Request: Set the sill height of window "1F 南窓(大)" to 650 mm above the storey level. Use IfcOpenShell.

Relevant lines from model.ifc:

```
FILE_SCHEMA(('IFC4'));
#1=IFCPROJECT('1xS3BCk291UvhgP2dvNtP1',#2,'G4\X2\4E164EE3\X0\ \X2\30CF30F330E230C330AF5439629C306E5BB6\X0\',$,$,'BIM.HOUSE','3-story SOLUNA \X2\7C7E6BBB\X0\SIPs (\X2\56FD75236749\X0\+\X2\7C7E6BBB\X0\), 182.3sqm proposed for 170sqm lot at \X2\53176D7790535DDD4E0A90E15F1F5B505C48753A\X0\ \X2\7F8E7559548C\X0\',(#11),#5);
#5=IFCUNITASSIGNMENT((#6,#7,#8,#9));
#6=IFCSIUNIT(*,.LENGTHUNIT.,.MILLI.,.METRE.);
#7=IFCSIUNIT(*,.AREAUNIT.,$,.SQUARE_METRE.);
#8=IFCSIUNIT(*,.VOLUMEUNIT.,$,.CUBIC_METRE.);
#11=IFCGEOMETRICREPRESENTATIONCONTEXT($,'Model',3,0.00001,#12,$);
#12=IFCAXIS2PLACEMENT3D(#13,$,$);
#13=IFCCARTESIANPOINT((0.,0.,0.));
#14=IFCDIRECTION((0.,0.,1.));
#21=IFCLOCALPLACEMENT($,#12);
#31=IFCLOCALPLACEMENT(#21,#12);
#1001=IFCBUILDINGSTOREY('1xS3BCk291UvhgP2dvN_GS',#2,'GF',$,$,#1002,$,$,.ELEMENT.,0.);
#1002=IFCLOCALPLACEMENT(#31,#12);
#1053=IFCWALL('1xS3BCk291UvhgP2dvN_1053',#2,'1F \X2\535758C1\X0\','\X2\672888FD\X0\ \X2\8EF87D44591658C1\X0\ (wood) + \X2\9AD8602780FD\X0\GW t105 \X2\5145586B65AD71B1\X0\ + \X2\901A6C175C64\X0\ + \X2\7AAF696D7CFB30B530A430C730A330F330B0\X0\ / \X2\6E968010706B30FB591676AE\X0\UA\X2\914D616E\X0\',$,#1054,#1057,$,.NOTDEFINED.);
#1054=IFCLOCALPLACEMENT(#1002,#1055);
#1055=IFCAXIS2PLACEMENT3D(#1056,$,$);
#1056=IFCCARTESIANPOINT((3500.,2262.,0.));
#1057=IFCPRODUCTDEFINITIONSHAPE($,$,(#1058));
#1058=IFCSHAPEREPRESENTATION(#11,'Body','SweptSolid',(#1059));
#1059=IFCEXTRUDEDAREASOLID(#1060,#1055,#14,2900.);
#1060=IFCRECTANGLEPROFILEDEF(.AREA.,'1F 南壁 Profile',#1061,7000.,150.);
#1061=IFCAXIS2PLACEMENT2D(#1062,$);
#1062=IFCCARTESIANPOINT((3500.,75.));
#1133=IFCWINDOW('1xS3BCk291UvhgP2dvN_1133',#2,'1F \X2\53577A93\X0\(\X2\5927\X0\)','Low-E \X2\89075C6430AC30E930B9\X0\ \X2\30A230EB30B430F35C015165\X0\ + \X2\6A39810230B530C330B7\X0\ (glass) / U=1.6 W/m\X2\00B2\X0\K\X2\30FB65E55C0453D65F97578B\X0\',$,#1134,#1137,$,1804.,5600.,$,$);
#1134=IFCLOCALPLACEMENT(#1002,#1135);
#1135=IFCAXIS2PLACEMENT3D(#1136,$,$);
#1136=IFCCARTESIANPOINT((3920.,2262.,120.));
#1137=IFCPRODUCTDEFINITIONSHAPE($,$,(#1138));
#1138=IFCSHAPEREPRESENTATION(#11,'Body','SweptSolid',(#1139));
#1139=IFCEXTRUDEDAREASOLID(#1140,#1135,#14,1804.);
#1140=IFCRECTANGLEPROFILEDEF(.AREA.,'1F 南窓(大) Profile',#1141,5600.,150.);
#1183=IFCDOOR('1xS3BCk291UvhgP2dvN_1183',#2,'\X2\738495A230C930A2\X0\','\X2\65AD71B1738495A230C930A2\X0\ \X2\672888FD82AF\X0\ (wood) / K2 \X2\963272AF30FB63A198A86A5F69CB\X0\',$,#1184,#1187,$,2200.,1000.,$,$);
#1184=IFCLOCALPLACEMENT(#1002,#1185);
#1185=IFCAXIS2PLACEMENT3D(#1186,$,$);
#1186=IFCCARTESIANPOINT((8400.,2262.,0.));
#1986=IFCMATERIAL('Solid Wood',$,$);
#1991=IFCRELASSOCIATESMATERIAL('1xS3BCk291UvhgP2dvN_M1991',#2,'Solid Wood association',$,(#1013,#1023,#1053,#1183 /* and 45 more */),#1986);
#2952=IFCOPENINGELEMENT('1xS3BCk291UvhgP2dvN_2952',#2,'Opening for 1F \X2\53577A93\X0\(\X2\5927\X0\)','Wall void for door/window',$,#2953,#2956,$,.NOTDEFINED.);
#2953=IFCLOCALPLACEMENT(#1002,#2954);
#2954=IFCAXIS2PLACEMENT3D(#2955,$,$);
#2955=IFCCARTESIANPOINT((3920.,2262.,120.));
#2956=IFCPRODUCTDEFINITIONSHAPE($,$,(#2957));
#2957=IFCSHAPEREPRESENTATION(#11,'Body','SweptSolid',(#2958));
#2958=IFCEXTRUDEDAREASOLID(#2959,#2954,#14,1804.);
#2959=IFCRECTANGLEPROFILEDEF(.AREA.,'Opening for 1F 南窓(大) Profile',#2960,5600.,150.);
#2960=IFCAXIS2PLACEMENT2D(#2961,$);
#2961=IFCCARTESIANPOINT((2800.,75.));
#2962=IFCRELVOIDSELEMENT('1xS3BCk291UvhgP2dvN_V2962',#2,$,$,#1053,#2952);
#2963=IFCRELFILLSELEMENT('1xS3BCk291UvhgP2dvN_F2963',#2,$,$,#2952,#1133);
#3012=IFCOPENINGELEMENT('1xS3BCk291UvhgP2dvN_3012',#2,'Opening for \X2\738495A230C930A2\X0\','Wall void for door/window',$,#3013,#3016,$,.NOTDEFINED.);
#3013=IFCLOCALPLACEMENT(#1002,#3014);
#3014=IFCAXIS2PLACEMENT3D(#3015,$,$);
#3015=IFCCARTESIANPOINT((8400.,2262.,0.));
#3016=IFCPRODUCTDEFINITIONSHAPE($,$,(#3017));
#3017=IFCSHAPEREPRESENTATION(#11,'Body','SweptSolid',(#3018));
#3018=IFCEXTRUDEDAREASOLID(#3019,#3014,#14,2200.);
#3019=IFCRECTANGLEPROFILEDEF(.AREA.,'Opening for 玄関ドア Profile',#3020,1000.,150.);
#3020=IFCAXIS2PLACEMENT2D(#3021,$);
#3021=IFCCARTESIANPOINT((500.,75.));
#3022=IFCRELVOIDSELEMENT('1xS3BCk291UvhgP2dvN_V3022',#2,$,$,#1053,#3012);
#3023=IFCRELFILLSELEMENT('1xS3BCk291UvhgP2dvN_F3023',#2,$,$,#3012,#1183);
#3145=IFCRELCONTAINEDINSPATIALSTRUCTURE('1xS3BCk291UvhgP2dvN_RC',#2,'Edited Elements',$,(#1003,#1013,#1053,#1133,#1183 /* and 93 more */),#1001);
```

```python
import numpy as np
import ifcopenshell
import ifcopenshell.api.geometry
import ifcopenshell.geom
import ifcopenshell.util.element
import ifcopenshell.util.placement
import ifcopenshell.util.shape
import ifcopenshell.util.unit

model = ifcopenshell.open("model.ifc")
unit_scale = ifcopenshell.util.unit.calculate_unit_scale(model)

window = model.by_guid("1xS3BCk291UvhgP2dvN_1133")
opening = window.FillsVoids[0].RelatingOpeningElement
storey = ifcopenshell.util.element.get_container(window, ifc_class="IfcBuildingStorey")
level = ifcopenshell.util.placement.get_local_placement(storey.ObjectPlacement)[2, 3]

# The opening's origin need not be at the sill, so measure its lowest point.
shape = ifcopenshell.geom.create_shape(ifcopenshell.geom.settings(), opening)
bottom = ifcopenshell.util.shape.get_shape_bottom_elevation(shape, shape.geometry) / unit_scale
dz = level + 0.65 / unit_scale - bottom

shift = np.array([0.0, 0.0, dz])
# The window is not placed relative to its opening, so move both.
for product in (opening, window):
    matrix = ifcopenshell.util.placement.get_local_placement(product.ObjectPlacement)
    matrix[:3, 3] += shift
    ifcopenshell.api.geometry.edit_object_placement(model, product=product, matrix=matrix, is_si=False)

print(f"moved by {dz * unit_scale:+.3f} m")

model.write("model_v2.ifc")
```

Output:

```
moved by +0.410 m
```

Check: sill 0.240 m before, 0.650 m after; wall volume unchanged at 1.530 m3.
